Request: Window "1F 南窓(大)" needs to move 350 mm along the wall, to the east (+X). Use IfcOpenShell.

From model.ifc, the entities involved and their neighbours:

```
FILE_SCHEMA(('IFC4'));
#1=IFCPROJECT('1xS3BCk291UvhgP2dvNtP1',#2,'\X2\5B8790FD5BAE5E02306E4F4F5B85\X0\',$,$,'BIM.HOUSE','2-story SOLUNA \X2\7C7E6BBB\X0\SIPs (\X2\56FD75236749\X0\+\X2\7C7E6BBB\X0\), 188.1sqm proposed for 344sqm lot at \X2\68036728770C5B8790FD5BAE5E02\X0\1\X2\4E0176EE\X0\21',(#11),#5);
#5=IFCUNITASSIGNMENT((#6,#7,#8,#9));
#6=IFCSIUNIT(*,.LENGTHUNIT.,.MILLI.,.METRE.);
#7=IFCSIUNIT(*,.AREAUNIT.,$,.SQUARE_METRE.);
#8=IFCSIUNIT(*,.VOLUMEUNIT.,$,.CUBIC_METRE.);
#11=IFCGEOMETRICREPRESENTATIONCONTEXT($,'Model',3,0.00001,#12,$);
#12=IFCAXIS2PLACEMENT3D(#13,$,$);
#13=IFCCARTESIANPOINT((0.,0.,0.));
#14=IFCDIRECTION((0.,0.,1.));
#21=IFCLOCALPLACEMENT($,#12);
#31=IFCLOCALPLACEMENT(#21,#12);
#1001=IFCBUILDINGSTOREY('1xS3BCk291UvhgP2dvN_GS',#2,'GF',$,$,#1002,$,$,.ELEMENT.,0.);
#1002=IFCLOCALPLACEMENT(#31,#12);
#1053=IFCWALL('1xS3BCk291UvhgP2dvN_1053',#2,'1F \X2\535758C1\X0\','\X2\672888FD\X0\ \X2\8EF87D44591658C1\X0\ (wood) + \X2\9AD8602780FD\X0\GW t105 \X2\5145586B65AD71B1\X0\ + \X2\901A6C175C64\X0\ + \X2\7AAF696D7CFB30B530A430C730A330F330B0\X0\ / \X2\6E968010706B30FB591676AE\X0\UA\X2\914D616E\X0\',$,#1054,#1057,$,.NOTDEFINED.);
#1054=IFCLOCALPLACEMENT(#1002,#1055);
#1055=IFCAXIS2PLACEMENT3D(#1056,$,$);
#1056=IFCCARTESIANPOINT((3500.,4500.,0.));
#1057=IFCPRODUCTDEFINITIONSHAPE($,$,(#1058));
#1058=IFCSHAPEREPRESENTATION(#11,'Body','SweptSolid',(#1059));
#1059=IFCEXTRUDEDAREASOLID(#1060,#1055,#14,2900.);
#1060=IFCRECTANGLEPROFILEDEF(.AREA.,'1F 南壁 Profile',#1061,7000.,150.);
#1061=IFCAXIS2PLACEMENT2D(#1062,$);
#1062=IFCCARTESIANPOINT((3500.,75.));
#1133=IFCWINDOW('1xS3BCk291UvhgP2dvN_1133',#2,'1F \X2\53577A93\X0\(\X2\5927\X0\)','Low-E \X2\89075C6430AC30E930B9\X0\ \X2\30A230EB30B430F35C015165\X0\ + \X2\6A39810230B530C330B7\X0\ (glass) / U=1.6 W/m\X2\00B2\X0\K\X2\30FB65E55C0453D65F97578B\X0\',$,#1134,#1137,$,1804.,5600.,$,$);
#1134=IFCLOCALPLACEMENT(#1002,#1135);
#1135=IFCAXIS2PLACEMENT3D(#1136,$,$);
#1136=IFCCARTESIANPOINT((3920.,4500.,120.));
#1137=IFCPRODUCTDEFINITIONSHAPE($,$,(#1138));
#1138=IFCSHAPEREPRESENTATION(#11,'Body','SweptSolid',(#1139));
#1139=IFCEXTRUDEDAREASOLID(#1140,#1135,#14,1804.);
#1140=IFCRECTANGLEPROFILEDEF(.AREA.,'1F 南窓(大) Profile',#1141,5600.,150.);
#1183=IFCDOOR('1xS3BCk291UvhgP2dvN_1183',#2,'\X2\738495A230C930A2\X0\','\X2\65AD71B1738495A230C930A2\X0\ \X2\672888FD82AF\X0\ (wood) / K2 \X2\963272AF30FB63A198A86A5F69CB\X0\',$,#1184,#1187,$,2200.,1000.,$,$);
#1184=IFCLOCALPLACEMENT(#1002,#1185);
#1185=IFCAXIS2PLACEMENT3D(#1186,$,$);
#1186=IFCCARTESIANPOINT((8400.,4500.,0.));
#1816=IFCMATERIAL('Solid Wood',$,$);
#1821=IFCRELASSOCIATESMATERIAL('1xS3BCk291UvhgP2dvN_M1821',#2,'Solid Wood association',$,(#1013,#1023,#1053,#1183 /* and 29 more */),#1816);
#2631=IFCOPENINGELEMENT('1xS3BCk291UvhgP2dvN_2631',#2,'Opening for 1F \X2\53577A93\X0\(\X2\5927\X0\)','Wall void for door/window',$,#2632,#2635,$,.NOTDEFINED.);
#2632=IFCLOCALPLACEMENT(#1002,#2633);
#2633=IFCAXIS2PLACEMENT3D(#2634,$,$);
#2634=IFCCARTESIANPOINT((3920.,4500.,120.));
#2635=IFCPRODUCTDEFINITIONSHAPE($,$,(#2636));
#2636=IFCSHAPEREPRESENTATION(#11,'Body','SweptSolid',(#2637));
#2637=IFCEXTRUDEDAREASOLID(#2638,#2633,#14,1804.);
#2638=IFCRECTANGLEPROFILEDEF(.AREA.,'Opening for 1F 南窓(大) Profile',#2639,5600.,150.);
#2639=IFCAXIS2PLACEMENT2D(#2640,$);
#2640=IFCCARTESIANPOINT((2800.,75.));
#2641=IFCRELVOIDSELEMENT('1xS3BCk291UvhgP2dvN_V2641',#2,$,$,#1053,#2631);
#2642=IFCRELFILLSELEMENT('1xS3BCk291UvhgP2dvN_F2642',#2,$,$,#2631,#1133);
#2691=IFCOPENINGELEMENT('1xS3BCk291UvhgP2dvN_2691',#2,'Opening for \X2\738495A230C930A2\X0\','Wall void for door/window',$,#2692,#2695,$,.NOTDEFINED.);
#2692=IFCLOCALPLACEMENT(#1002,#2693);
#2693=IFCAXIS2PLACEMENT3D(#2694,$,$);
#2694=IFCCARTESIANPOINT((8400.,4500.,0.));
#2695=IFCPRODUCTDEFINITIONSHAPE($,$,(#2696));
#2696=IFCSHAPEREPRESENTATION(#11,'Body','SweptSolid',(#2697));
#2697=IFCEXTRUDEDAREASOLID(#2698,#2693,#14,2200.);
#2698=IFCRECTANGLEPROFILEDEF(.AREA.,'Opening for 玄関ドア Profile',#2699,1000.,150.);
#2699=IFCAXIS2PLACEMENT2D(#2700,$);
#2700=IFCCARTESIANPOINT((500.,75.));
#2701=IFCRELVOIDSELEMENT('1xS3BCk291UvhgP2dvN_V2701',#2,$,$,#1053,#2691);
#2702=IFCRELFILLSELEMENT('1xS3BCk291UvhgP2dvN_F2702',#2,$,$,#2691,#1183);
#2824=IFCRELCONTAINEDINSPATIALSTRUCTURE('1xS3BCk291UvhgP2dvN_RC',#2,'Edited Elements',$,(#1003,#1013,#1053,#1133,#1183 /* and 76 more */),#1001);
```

```python
import ifcopenshell
import ifcopenshell.api.geometry
import ifcopenshell.util.placement

model = ifcopenshell.open("model.ifc")

window = model.by_id(1133)
opening = window.FillsVoids[0].RelatingOpeningElement
wall = opening.VoidsElements[0].RelatingBuildingElement

wall_matrix = ifcopenshell.util.placement.get_local_placement(wall.ObjectPlacement)
shift = wall_matrix[:3, 0] * 350.0
before = ifcopenshell.util.placement.get_local_placement(window.ObjectPlacement)[:3, 3].copy()

# The window is not placed relative to its opening, so move both.
for product in (opening, window):
    matrix = ifcopenshell.util.placement.get_local_placement(product.ObjectPlacement)
    matrix[:3, 3] += shift
    ifcopenshell.api.geometry.edit_object_placement(model, product=product, matrix=matrix, is_si=False)

after = ifcopenshell.util.placement.get_local_placement(window.ObjectPlacement)[:3, 3]
print("window moved by", (after - before).round(3) + 0.0)

model.write("model-out.ifc")
```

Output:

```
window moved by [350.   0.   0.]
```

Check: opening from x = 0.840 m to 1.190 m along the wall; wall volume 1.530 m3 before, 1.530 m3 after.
